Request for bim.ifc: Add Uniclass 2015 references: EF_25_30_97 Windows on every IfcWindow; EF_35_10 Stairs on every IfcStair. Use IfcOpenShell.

First a look at what the model holds.

```python
import ifcopenshell

model = ifcopenshell.open("bim.ifc")
print(model.schema)
print("classifications:", [c.Name for c in model.by_type("IfcClassification")])
for ifc_class in ("IfcDoor", "IfcRoof", "IfcStair", "IfcWall", "IfcWindow"):
    print(ifc_class, len(model.by_type(ifc_class)))
```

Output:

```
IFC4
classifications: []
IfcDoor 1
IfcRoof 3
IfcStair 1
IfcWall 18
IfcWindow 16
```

```python
import ifcopenshell
import ifcopenshell.api.classification

model = ifcopenshell.open("bim.ifc")

system = ifcopenshell.api.classification.add_classification(model, classification="Uniclass 2015")

codes = {
    "IfcWindow": ("EF_25_30_97", "Windows"),
    "IfcStair": ("EF_35_10", "Stairs"),
}
for ifc_class, (code, name) in codes.items():
    products = model.by_type(ifc_class)
    ifcopenshell.api.classification.add_reference(
        model, products=products, classification=system, identification=code, name=name
    )
    print(code, len(products))

model.write("bim_updated.ifc")
```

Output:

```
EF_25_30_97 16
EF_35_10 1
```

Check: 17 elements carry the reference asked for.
